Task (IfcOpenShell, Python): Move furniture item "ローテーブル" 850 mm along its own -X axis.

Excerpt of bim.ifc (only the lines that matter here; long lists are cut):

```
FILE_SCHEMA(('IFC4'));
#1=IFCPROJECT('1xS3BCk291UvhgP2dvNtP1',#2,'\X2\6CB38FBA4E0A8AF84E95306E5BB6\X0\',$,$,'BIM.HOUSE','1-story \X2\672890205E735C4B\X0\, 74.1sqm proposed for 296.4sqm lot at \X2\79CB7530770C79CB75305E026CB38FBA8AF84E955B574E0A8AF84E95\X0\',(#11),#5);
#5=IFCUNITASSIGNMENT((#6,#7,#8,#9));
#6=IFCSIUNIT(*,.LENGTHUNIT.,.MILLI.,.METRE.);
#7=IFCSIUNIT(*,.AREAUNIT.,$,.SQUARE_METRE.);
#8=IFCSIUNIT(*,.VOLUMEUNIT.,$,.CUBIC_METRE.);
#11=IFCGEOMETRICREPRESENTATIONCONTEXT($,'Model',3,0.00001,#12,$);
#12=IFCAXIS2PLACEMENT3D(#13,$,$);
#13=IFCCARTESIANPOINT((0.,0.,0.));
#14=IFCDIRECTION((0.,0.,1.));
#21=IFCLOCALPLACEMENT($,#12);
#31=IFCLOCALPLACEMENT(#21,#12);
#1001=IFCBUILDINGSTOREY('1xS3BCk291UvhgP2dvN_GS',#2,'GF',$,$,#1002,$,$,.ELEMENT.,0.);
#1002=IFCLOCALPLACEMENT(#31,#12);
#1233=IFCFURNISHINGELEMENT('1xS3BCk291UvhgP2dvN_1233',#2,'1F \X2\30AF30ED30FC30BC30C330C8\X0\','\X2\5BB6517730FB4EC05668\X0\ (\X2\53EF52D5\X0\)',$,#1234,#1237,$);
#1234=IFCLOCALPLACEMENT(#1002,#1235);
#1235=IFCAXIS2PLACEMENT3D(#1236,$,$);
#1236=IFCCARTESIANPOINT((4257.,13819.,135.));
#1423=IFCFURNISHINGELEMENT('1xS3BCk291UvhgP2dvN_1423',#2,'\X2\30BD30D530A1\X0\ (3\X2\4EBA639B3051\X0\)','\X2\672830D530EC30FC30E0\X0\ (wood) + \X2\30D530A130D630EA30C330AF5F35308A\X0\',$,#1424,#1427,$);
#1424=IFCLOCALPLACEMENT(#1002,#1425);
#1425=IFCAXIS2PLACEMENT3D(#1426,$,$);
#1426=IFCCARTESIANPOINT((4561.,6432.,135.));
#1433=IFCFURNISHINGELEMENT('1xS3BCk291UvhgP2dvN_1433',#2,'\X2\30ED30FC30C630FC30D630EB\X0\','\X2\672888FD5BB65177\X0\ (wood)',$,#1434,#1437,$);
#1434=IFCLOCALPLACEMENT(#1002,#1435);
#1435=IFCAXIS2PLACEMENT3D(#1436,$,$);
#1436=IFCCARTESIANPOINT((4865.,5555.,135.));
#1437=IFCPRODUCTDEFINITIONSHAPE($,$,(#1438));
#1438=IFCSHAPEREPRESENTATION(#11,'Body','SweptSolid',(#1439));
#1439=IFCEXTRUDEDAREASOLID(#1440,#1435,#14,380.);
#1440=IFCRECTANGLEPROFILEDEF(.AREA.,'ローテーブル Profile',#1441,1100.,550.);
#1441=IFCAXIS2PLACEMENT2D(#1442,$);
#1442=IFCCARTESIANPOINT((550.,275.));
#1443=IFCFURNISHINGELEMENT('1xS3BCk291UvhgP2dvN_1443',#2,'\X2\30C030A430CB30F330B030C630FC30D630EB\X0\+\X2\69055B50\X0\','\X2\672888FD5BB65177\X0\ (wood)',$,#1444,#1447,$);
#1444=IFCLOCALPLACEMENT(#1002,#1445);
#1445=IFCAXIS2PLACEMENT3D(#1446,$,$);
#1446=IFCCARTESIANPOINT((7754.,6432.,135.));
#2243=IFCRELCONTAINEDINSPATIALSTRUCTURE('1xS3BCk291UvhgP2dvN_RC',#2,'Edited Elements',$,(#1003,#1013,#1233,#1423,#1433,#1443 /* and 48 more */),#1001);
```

```python
import ifcopenshell
import ifcopenshell.api.geometry
import ifcopenshell.util.placement
import ifcopenshell.util.unit

model = ifcopenshell.open("bim.ifc")
unit_scale = ifcopenshell.util.unit.calculate_unit_scale(model)

item = model.by_id(1433)
matrix = ifcopenshell.util.placement.get_local_placement(item.ObjectPlacement)
matrix[:3, 3] -= matrix[:3, 0] * 0.85 / unit_scale
ifcopenshell.api.geometry.edit_object_placement(model, product=item, matrix=matrix, is_si=False)

print(ifcopenshell.util.placement.get_local_placement(item.ObjectPlacement).round(3) + 0.0)

model.write("bim_rev.ifc")
```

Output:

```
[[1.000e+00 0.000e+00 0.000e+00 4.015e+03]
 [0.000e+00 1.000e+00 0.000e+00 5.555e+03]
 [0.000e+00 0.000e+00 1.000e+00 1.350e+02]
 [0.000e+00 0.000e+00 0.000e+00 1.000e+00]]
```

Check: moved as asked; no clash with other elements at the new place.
